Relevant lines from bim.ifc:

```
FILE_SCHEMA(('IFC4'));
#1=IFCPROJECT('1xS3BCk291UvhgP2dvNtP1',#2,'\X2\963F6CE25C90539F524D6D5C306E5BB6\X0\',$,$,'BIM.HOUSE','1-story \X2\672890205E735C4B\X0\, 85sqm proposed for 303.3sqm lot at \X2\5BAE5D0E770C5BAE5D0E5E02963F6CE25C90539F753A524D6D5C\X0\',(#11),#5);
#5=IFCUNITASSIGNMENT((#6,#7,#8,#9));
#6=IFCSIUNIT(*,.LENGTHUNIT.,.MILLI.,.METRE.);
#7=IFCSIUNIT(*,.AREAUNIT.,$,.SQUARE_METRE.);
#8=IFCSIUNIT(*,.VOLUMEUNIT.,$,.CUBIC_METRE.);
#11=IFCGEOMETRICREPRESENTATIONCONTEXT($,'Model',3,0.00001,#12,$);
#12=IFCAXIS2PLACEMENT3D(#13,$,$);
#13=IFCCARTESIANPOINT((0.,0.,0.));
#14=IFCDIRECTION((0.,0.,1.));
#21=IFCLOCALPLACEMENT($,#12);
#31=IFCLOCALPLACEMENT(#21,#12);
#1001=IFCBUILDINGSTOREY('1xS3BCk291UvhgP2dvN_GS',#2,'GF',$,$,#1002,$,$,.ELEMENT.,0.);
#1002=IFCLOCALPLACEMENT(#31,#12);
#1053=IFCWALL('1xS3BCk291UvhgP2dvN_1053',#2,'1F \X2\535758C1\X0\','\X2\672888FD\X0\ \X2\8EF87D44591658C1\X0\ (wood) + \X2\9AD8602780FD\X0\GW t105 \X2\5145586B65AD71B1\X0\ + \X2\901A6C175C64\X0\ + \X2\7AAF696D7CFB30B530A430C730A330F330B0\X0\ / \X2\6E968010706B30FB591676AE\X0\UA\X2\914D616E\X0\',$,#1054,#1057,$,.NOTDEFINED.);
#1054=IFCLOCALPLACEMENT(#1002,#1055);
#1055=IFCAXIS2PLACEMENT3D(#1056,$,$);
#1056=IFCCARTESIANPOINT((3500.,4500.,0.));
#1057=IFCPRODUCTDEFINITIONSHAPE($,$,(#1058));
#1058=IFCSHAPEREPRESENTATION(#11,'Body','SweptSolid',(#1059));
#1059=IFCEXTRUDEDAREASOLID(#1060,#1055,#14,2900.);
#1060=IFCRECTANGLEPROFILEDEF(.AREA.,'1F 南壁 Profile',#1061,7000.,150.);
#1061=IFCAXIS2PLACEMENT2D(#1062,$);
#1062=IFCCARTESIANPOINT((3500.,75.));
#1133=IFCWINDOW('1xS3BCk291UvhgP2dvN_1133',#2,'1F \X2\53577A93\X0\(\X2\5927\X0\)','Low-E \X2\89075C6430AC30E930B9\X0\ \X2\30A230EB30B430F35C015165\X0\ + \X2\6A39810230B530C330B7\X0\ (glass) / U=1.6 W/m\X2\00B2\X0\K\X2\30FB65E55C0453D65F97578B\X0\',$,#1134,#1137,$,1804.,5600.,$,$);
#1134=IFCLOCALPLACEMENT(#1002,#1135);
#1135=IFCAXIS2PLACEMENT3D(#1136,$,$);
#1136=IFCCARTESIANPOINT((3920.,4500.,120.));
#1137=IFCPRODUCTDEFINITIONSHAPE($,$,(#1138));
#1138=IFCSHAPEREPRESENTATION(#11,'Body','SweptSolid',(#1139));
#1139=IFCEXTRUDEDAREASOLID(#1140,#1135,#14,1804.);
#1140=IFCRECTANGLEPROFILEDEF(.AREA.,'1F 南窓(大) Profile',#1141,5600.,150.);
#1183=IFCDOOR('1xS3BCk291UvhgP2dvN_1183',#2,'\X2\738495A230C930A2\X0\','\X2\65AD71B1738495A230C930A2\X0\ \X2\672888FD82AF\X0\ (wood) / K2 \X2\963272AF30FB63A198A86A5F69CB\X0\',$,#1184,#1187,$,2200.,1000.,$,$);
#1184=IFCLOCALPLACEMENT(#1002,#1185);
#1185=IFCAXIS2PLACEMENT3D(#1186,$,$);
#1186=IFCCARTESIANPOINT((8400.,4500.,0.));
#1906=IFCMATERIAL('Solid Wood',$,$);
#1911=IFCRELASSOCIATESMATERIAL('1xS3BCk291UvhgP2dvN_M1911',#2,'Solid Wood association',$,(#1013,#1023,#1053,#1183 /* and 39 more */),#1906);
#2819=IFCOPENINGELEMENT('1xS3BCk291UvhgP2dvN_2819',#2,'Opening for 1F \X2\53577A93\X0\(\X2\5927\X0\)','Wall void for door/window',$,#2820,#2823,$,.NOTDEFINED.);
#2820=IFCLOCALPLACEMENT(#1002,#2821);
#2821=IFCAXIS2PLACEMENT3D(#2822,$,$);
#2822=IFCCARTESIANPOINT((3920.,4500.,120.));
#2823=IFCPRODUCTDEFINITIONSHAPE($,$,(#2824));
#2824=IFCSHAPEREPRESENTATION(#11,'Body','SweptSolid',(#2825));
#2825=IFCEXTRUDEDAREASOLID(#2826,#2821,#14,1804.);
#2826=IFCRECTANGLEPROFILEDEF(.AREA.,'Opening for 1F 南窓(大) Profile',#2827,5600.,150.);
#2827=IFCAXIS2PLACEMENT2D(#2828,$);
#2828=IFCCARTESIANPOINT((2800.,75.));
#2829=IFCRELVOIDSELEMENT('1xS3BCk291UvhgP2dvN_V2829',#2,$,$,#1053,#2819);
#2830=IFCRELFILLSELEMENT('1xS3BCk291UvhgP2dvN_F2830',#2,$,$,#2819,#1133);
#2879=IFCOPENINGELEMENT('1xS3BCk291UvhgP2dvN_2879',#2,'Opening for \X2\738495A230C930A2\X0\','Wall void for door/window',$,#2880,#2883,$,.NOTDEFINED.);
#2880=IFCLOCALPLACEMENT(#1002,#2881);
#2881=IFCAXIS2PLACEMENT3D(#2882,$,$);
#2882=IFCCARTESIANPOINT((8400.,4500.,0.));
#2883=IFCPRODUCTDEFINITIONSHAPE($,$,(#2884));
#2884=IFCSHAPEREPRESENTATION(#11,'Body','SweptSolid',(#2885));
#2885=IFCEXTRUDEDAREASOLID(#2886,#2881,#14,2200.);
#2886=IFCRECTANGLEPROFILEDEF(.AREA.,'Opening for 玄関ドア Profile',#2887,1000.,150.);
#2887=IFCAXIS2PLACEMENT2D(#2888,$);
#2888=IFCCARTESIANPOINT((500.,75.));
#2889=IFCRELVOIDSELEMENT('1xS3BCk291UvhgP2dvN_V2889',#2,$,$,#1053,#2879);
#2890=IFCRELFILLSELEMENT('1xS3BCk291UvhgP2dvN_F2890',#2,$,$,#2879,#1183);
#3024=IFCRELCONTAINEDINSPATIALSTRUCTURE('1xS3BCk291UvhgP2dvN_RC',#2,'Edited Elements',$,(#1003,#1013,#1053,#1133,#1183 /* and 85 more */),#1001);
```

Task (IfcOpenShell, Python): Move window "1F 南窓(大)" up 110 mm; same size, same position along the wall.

```python
import numpy as np
import ifcopenshell
import ifcopenshell.api.geometry
import ifcopenshell.util.placement
import ifcopenshell.util.unit

model = ifcopenshell.open("bim.ifc")
unit_scale = ifcopenshell.util.unit.calculate_unit_scale(model)

window = model.by_guid("1xS3BCk291UvhgP2dvN_1133")
opening = window.FillsVoids[0].RelatingOpeningElement
dz = 110.0

shift = np.array([0.0, 0.0, dz])
# The window is not placed relative to its opening, so move both.
for product in (opening, window):
    matrix = ifcopenshell.util.placement.get_local_placement(product.ObjectPlacement)
    matrix[:3, 3] += shift
    ifcopenshell.api.geometry.edit_object_placement(model, product=product, matrix=matrix, is_si=False)

print(f"moved by {dz * unit_scale:+.3f} m")

model.write("bim_updated.ifc")
```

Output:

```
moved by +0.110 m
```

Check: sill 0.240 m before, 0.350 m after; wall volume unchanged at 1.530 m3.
